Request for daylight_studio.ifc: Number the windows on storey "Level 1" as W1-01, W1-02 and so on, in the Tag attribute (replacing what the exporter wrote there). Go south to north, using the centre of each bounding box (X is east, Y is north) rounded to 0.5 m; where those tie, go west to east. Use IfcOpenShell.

First a look at what the model holds.

```python
import ifcopenshell
import ifcopenshell.util.element
import ifcopenshell.util.placement

model = ifcopenshell.open("daylight_studio.ifc")
print(model.schema)
storey = next(s for s in model.by_type("IfcBuildingStorey") if s.Name == "Level 1")
windows = [e for e in ifcopenshell.util.element.get_decomposition(storey) if e.is_a("IfcWindow")]
for e in sorted(windows, key=lambda e: e.id()):
    origin = ifcopenshell.util.placement.get_local_placement(e.ObjectPlacement)[:3, 3]
    print(e.id(), e.Tag, e.Name, origin.round(2) + 0.0, sep=" | ")
```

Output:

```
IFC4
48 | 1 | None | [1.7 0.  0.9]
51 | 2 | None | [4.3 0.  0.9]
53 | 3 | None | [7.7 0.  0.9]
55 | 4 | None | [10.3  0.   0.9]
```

```python
import ifcopenshell
import ifcopenshell.geom
import ifcopenshell.util.element
import ifcopenshell.util.shape

model = ifcopenshell.open("daylight_studio.ifc")
settings = ifcopenshell.geom.settings()
settings.set("use-world-coords", True)


def centre(element):
    shape = ifcopenshell.geom.create_shape(settings, element)
    return ifcopenshell.util.shape.get_bbox_centroid(shape.geometry)


storey = next(s for s in model.by_type("IfcBuildingStorey") if s.Name == "Level 1")
windows = [e for e in ifcopenshell.util.element.get_decomposition(storey) if e.is_a("IfcWindow")]

# Insertion points can sit at a corner or the storey origin, so sort by the geometry (in metres).
centres = {e: centre(e) for e in windows}
windows.sort(key=lambda e: (round(centres[e][1] / 0.5), centres[e][0]))

for i, e in enumerate(windows, start=1):
    number = f"W1-{i:02d}"
    e.Tag = number
    print(e.id(), number)

model.write("daylight_studio_v2.ifc")
```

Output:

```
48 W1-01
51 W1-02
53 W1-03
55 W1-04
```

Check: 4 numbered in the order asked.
